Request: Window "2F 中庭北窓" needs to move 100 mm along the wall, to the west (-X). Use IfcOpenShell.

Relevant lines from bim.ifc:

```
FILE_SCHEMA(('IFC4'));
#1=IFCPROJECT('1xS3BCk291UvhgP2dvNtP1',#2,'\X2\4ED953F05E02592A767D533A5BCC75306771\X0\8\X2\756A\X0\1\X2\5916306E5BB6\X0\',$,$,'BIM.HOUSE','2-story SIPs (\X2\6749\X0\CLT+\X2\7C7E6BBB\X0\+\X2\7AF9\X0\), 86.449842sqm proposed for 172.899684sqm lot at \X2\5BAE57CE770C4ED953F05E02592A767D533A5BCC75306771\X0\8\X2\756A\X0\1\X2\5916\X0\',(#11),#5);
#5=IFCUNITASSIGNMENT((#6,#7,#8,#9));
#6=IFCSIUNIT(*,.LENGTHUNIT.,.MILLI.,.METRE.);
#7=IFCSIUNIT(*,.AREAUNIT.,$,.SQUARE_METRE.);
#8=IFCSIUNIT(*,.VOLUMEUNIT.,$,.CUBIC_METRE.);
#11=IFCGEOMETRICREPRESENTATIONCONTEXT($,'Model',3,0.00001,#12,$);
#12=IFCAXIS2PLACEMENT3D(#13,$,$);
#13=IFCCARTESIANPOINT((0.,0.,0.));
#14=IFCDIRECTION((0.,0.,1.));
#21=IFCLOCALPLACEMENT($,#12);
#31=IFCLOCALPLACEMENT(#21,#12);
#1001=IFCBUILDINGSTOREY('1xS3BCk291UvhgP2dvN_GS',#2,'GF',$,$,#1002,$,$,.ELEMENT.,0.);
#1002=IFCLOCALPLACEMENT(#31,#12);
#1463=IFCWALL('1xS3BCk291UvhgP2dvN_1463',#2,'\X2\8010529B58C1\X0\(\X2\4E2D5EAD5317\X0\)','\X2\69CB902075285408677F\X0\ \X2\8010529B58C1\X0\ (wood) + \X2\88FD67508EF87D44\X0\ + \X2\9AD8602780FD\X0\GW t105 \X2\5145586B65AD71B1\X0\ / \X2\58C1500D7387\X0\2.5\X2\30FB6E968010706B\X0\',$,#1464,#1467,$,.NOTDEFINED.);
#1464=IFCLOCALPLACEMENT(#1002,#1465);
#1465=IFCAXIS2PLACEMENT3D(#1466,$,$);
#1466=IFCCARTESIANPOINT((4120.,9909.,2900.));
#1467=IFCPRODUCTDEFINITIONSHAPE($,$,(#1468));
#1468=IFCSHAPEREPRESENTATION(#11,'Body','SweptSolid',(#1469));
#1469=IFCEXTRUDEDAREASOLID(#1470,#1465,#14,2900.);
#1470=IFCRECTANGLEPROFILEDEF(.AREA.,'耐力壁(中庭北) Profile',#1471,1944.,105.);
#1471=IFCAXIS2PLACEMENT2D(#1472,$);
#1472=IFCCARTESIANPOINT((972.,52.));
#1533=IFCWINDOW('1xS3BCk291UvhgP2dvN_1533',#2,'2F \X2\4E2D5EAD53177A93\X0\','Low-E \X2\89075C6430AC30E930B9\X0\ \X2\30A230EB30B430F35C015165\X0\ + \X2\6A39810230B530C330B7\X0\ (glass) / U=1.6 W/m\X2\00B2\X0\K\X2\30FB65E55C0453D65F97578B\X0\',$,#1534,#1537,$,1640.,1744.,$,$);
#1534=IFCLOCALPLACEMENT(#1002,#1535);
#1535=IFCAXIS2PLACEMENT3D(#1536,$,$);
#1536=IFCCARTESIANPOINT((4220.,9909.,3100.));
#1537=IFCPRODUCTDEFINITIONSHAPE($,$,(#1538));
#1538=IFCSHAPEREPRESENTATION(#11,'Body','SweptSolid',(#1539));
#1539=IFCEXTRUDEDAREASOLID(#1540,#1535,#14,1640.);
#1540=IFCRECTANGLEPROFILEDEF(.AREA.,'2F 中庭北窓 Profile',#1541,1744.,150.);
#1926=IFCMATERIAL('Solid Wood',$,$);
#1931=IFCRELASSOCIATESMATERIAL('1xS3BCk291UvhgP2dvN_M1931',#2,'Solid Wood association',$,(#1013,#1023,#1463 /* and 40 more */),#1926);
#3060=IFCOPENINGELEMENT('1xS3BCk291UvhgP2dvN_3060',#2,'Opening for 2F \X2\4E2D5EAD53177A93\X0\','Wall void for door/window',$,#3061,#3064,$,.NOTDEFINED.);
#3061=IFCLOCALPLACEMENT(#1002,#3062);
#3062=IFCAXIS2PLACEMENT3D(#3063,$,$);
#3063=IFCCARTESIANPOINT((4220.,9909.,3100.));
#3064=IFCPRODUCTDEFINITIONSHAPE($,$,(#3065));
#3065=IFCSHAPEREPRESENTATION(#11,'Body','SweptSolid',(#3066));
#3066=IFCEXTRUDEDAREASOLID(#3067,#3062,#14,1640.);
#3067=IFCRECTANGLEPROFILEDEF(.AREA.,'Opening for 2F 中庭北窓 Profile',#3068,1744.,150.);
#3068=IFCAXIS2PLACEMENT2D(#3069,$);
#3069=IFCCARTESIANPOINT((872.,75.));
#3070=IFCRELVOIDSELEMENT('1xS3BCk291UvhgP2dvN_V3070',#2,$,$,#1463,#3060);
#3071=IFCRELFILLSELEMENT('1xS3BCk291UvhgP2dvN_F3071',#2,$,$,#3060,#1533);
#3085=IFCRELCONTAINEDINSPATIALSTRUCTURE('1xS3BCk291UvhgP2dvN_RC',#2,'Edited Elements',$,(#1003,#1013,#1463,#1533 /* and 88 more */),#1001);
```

```python
import ifcopenshell
import ifcopenshell.api.geometry
import ifcopenshell.util.placement

model = ifcopenshell.open("bim.ifc")

window = model.by_id(1533)
opening = window.FillsVoids[0].RelatingOpeningElement
wall = opening.VoidsElements[0].RelatingBuildingElement

wall_matrix = ifcopenshell.util.placement.get_local_placement(wall.ObjectPlacement)
shift = wall_matrix[:3, 0] * -100.0
before = ifcopenshell.util.placement.get_local_placement(window.ObjectPlacement)[:3, 3].copy()

# The window is not placed relative to its opening, so move both.
for product in (opening, window):
    matrix = ifcopenshell.util.placement.get_local_placement(product.ObjectPlacement)
    matrix[:3, 3] += shift
    ifcopenshell.api.geometry.edit_object_placement(model, product=product, matrix=matrix, is_si=False)

after = ifcopenshell.util.placement.get_local_placement(window.ObjectPlacement)[:3, 3]
print("window moved by", (after - before).round(3) + 0.0)

model.write("bim-out.ifc")
```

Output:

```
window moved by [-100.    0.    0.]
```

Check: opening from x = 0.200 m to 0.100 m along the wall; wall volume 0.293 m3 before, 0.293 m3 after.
